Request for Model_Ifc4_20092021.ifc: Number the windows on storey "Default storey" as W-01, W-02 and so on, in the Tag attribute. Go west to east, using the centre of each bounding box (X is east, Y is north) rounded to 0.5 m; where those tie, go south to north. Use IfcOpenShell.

First a look at what the model holds.

```python
import ifcopenshell
import ifcopenshell.util.element
import ifcopenshell.util.placement

model = ifcopenshell.open("Model_Ifc4_20092021.ifc")
print(model.schema)
storey = next(s for s in model.by_type("IfcBuildingStorey") if s.Name == "Default storey")
windows = [e for e in ifcopenshell.util.element.get_decomposition(storey) if e.is_a("IfcWindow")]
for e in sorted(windows, key=lambda e: e.id()):
    origin = ifcopenshell.util.placement.get_local_placement(e.ObjectPlacement)[:3, 3]
    print(e.id(), e.Tag, e.Name, origin.round(2) + 0.0, sep=" | ")
```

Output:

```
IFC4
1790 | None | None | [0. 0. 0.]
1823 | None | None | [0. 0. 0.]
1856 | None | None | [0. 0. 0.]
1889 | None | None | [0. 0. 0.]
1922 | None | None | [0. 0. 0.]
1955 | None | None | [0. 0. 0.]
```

```python
import ifcopenshell
import ifcopenshell.geom
import ifcopenshell.util.element
import ifcopenshell.util.shape

model = ifcopenshell.open("Model_Ifc4_20092021.ifc")
settings = ifcopenshell.geom.settings()
settings.set("use-world-coords", True)


def centre(element):
    shape = ifcopenshell.geom.create_shape(settings, element)
    return ifcopenshell.util.shape.get_bbox_centroid(shape.geometry)


storey = next(s for s in model.by_type("IfcBuildingStorey") if s.Name == "Default storey")
windows = [e for e in ifcopenshell.util.element.get_decomposition(storey) if e.is_a("IfcWindow")]

# Insertion points can sit at a corner or the storey origin, so sort by the geometry (in metres).
centres = {e: centre(e) for e in windows}
windows.sort(key=lambda e: (round(centres[e][0] / 0.5), centres[e][1]))

for i, e in enumerate(windows, start=1):
    number = f"W-{i:02d}"
    e.Tag = number
    print(e.id(), number)

model.write("Model_Ifc4_20092021_v2.ifc")
```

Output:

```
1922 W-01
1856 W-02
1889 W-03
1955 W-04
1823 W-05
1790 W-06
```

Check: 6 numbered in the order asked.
